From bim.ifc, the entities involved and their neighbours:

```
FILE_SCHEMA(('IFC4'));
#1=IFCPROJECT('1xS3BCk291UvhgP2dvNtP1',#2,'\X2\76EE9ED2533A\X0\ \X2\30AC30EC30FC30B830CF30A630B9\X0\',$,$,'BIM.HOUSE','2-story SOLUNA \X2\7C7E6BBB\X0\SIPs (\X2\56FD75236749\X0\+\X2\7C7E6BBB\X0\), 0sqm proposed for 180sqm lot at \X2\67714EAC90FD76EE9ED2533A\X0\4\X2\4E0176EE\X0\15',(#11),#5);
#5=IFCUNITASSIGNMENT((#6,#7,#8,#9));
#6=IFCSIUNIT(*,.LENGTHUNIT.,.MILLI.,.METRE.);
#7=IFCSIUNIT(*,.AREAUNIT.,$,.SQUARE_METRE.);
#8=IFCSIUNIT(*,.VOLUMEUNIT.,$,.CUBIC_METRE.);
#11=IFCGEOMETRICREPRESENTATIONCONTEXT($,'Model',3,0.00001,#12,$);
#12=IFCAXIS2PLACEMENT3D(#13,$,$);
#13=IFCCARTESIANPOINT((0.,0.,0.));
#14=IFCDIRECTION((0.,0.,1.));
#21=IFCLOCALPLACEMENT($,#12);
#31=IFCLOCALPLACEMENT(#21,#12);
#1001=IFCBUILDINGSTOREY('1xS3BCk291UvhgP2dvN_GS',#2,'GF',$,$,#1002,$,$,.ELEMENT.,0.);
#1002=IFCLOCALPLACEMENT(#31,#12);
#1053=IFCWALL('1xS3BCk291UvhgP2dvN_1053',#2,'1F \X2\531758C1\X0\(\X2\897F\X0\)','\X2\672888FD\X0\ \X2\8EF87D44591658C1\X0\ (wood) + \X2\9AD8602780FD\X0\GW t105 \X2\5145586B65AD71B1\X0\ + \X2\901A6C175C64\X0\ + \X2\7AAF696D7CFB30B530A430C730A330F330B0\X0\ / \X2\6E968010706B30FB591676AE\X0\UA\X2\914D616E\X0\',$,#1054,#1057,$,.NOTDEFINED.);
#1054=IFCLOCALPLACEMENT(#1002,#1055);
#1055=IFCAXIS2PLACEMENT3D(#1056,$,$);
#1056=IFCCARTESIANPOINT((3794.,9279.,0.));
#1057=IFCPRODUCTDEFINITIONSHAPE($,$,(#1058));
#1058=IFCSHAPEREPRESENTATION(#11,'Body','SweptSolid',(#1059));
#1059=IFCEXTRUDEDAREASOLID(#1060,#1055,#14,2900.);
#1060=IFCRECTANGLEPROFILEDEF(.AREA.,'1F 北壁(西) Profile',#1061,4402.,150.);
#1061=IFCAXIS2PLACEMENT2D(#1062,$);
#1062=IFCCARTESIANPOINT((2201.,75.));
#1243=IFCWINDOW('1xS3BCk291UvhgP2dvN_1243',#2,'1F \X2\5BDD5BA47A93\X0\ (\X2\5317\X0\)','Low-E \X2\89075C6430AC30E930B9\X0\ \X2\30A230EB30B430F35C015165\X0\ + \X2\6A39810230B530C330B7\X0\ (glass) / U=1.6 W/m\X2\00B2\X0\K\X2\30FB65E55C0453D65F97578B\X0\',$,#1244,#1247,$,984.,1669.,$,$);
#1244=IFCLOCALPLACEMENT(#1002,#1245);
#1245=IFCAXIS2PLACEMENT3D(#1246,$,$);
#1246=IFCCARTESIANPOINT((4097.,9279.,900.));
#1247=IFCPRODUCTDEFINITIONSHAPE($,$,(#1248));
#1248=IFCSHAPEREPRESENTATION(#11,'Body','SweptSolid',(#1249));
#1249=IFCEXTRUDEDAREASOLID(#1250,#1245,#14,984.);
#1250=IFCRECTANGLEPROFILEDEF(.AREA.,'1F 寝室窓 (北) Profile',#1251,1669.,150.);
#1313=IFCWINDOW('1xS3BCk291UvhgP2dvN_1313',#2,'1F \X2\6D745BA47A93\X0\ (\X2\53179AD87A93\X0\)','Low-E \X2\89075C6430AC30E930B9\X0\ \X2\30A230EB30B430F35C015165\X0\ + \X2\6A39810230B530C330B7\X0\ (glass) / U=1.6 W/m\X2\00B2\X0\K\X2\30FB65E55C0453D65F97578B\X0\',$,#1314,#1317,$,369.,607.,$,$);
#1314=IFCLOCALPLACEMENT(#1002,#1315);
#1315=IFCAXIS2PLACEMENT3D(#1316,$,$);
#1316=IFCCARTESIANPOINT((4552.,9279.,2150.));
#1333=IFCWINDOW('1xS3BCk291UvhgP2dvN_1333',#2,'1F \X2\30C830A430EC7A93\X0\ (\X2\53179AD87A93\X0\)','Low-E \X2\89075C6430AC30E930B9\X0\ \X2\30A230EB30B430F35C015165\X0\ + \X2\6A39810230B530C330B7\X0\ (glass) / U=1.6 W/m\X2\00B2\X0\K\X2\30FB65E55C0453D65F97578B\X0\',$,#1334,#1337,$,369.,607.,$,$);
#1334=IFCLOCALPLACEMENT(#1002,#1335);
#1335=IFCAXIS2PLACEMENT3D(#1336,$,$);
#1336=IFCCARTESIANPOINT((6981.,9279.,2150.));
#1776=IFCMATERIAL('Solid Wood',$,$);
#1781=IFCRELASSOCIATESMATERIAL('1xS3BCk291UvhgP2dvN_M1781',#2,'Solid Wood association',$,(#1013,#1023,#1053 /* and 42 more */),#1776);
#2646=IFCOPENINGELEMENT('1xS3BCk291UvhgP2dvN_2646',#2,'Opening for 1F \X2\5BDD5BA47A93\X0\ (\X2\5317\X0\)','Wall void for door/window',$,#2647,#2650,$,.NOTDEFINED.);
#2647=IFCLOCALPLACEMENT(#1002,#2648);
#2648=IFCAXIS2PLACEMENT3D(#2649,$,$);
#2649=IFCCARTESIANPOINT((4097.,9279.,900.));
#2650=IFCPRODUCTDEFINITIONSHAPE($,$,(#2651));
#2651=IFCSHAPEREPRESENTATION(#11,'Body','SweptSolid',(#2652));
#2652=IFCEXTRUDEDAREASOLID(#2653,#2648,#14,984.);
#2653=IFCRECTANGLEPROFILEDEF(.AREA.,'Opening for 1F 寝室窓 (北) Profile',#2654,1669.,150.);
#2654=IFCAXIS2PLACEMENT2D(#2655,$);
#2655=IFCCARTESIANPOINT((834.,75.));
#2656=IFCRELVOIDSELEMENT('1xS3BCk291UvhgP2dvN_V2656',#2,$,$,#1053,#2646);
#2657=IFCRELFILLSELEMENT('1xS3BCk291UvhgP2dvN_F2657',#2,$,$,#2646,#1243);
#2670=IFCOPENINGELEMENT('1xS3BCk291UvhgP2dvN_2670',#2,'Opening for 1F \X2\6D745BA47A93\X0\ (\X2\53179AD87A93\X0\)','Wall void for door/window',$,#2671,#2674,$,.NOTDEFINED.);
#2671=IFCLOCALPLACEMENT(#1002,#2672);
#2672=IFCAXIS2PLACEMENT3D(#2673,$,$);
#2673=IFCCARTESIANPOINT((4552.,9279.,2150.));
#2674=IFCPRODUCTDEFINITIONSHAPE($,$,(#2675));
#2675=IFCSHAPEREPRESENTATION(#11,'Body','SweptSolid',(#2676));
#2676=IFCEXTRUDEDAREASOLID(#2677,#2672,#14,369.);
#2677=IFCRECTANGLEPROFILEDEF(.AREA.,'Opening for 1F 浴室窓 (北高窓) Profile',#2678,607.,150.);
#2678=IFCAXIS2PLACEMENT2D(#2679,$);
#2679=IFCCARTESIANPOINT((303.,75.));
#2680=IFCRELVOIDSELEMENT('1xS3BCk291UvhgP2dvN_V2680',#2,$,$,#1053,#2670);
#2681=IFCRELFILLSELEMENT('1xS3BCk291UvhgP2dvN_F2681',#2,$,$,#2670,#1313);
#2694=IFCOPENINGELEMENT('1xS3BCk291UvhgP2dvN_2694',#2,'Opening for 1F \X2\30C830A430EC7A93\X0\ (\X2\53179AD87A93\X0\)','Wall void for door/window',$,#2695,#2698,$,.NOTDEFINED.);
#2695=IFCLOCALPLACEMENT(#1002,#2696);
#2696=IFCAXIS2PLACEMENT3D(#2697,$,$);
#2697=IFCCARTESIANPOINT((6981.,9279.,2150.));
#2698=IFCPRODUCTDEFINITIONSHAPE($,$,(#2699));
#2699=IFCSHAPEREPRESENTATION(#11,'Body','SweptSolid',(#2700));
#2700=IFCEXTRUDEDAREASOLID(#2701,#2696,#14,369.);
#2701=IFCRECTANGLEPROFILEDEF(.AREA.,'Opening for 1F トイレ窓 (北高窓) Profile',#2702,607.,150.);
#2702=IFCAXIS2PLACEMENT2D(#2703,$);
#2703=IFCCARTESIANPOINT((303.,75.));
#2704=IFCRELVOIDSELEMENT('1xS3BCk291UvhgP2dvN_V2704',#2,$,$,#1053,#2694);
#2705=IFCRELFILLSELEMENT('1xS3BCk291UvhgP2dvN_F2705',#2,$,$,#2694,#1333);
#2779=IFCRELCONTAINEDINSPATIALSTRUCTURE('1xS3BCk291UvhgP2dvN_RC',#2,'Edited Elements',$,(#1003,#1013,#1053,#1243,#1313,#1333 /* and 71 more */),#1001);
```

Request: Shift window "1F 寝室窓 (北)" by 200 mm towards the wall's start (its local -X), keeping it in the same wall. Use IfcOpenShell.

```python
import ifcopenshell
import ifcopenshell.api.geometry
import ifcopenshell.util.placement

model = ifcopenshell.open("bim.ifc")

window = model.by_guid("1xS3BCk291UvhgP2dvN_1243")
opening = window.FillsVoids[0].RelatingOpeningElement
wall = opening.VoidsElements[0].RelatingBuildingElement

wall_matrix = ifcopenshell.util.placement.get_local_placement(wall.ObjectPlacement)
shift = wall_matrix[:3, 0] * -200.0
before = ifcopenshell.util.placement.get_local_placement(window.ObjectPlacement)[:3, 3].copy()

# The window is not placed relative to its opening, so move both.
for product in (opening, window):
    matrix = ifcopenshell.util.placement.get_local_placement(product.ObjectPlacement)
    matrix[:3, 3] += shift
    ifcopenshell.api.geometry.edit_object_placement(model, product=product, matrix=matrix, is_si=False)

after = ifcopenshell.util.placement.get_local_placement(window.ObjectPlacement)[:3, 3]
print("window moved by", (after - before).round(3) + 0.0)

model.write("bim_v2.ifc")
```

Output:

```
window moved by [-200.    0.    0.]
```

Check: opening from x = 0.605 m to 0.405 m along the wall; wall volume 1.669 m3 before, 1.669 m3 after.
